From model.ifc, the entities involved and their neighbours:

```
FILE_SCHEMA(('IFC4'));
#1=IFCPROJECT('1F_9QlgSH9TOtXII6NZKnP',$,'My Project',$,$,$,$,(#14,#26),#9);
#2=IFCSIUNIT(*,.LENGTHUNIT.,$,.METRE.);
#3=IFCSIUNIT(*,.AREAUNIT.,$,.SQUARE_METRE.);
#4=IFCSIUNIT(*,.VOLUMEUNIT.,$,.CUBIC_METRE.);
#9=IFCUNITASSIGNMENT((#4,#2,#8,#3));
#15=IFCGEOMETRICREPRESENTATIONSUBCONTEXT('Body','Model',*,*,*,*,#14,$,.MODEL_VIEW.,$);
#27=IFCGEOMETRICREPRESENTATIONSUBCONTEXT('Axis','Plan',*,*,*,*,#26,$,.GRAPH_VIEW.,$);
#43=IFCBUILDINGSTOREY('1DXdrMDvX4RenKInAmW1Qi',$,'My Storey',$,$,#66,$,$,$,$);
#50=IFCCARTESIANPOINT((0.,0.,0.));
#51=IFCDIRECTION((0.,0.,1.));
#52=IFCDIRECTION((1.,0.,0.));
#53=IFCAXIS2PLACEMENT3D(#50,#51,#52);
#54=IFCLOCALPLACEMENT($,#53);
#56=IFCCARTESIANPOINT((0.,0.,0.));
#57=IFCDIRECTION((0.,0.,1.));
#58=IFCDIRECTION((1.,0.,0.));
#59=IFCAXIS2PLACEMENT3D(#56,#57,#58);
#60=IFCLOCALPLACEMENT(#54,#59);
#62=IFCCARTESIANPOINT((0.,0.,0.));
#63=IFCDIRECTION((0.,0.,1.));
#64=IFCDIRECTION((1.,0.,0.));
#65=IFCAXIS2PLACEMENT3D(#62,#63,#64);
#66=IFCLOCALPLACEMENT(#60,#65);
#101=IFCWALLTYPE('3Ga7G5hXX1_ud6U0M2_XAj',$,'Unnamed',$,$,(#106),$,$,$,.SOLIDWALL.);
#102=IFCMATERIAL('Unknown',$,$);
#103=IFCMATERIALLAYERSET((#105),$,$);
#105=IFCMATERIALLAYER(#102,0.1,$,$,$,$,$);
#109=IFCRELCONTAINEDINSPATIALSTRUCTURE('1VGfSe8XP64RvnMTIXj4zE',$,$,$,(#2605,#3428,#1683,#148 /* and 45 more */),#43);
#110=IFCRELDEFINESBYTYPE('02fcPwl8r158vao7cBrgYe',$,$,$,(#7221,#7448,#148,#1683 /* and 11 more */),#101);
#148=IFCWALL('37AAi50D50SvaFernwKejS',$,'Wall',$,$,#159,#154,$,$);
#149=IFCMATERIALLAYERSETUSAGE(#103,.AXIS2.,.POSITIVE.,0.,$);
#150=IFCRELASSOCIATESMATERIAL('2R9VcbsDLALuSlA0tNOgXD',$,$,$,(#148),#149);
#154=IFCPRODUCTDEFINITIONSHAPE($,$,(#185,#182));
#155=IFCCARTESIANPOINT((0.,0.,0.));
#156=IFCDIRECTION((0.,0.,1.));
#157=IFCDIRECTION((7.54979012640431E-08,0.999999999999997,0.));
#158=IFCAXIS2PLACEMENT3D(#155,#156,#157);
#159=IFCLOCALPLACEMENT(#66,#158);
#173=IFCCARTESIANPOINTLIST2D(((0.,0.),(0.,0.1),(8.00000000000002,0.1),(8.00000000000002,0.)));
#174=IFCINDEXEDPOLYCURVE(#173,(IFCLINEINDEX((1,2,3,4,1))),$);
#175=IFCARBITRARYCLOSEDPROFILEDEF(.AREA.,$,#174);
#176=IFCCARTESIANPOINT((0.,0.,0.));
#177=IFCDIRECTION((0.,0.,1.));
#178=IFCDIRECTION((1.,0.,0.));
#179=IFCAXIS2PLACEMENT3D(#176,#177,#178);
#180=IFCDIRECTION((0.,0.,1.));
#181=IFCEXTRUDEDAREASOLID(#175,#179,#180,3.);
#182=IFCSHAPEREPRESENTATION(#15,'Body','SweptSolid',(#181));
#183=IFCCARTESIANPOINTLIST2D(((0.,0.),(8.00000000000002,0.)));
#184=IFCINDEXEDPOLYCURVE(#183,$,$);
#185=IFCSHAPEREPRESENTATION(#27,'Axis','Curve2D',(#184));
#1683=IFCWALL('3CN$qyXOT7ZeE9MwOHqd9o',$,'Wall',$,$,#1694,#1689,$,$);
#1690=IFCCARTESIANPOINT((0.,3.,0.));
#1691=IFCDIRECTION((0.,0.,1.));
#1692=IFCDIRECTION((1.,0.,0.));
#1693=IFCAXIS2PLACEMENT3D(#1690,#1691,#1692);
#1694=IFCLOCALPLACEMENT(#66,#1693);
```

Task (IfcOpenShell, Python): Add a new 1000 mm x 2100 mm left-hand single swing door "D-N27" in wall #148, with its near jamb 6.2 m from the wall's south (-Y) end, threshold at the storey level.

```python
import numpy as np
import ifcopenshell
import ifcopenshell.api.feature
import ifcopenshell.api.geometry
import ifcopenshell.api.root
import ifcopenshell.api.spatial
import ifcopenshell.geom
import ifcopenshell.util.element
import ifcopenshell.util.placement
import ifcopenshell.util.representation
import ifcopenshell.util.shape
import ifcopenshell.util.unit

model = ifcopenshell.open("model.ifc")
unit_scale = ifcopenshell.util.unit.calculate_unit_scale(model)
settings = ifcopenshell.geom.settings()


def volume(element):
    """Net volume in cubic metres, openings subtracted."""
    shape = ifcopenshell.geom.create_shape(settings, element)
    return ifcopenshell.util.shape.get_volume(shape.geometry)


wall = model.by_guid("37AAi50D50SvaFernwKejS")
storey = ifcopenshell.util.element.get_container(wall, ifc_class="IfcBuildingStorey")
context = ifcopenshell.util.representation.get_context(model, "Model", "Body", "MODEL_VIEW")
before = volume(wall)

width, height, from_end, sill = 1, 2.1, 6.2, 0.0  # metres

# The wall runs along its own X axis, and the end named is its -X end.
wall_shape = ifcopenshell.geom.create_shape(settings, wall)
x, y, z = ifcopenshell.util.shape.get_vertices(wall_shape.geometry).T
start = x.min() + from_end
face, thickness = float(y.min()), float(y.max() - y.min())
wall_matrix = ifcopenshell.util.placement.get_local_placement(wall.ObjectPlacement)
level = ifcopenshell.util.placement.get_local_placement(storey.ObjectPlacement)[2, 3]


def in_wall(x, y):
    """Placement at x, y metres in the wall's axes, at sill height."""
    matrix = wall_matrix.copy()
    matrix[:, 3] = wall_matrix @ np.array([x / unit_scale, y / unit_scale, 0.0, 1.0])
    matrix[2, 3] = level + sill / unit_scale
    return matrix


# Opening: a box that overshoots both wall faces by 50 mm.
opening = ifcopenshell.api.root.create_entity(model, ifc_class="IfcOpeningElement", predefined_type="OPENING")
box = ifcopenshell.api.geometry.add_wall_representation(
    model, context=context, length=width, height=height, thickness=thickness + 0.1
)
ifcopenshell.api.geometry.assign_representation(model, product=opening, representation=box)
ifcopenshell.api.geometry.edit_object_placement(model, product=opening, matrix=in_wall(start, face - 0.05), is_si=False)
ifcopenshell.api.feature.add_feature(model, feature=opening, element=wall)

door = ifcopenshell.api.root.create_entity(model, ifc_class="IfcDoor", name="D-N27", predefined_type="DOOR")
door.OverallWidth, door.OverallHeight = width / unit_scale, height / unit_scale
door.OperationType = "SINGLE_SWING_LEFT"
body = ifcopenshell.api.geometry.add_door_representation(
    model,
    context=context,
    overall_width=door.OverallWidth,
    overall_height=door.OverallHeight,
    operation_type="SINGLE_SWING_LEFT",
    lining_properties={"LiningDepth": thickness / unit_scale, "ThresholdDepth": thickness / unit_scale},
)
ifcopenshell.api.geometry.assign_representation(model, product=door, representation=body)
ifcopenshell.api.spatial.assign_container(model, products=[door], relating_structure=storey)
ifcopenshell.api.feature.add_filling(model, opening=opening, element=door)

# The lining spans the wall, so the door starts at the wall face.
ifcopenshell.api.geometry.edit_object_placement(model, product=door, matrix=in_wall(start, face), is_si=False)

after = volume(wall)

print(f"wall volume {before:.3f} -> {after:.3f} m3")

model.write("model_updated.ifc")
```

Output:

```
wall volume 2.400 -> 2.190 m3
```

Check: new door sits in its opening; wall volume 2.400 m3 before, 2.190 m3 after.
